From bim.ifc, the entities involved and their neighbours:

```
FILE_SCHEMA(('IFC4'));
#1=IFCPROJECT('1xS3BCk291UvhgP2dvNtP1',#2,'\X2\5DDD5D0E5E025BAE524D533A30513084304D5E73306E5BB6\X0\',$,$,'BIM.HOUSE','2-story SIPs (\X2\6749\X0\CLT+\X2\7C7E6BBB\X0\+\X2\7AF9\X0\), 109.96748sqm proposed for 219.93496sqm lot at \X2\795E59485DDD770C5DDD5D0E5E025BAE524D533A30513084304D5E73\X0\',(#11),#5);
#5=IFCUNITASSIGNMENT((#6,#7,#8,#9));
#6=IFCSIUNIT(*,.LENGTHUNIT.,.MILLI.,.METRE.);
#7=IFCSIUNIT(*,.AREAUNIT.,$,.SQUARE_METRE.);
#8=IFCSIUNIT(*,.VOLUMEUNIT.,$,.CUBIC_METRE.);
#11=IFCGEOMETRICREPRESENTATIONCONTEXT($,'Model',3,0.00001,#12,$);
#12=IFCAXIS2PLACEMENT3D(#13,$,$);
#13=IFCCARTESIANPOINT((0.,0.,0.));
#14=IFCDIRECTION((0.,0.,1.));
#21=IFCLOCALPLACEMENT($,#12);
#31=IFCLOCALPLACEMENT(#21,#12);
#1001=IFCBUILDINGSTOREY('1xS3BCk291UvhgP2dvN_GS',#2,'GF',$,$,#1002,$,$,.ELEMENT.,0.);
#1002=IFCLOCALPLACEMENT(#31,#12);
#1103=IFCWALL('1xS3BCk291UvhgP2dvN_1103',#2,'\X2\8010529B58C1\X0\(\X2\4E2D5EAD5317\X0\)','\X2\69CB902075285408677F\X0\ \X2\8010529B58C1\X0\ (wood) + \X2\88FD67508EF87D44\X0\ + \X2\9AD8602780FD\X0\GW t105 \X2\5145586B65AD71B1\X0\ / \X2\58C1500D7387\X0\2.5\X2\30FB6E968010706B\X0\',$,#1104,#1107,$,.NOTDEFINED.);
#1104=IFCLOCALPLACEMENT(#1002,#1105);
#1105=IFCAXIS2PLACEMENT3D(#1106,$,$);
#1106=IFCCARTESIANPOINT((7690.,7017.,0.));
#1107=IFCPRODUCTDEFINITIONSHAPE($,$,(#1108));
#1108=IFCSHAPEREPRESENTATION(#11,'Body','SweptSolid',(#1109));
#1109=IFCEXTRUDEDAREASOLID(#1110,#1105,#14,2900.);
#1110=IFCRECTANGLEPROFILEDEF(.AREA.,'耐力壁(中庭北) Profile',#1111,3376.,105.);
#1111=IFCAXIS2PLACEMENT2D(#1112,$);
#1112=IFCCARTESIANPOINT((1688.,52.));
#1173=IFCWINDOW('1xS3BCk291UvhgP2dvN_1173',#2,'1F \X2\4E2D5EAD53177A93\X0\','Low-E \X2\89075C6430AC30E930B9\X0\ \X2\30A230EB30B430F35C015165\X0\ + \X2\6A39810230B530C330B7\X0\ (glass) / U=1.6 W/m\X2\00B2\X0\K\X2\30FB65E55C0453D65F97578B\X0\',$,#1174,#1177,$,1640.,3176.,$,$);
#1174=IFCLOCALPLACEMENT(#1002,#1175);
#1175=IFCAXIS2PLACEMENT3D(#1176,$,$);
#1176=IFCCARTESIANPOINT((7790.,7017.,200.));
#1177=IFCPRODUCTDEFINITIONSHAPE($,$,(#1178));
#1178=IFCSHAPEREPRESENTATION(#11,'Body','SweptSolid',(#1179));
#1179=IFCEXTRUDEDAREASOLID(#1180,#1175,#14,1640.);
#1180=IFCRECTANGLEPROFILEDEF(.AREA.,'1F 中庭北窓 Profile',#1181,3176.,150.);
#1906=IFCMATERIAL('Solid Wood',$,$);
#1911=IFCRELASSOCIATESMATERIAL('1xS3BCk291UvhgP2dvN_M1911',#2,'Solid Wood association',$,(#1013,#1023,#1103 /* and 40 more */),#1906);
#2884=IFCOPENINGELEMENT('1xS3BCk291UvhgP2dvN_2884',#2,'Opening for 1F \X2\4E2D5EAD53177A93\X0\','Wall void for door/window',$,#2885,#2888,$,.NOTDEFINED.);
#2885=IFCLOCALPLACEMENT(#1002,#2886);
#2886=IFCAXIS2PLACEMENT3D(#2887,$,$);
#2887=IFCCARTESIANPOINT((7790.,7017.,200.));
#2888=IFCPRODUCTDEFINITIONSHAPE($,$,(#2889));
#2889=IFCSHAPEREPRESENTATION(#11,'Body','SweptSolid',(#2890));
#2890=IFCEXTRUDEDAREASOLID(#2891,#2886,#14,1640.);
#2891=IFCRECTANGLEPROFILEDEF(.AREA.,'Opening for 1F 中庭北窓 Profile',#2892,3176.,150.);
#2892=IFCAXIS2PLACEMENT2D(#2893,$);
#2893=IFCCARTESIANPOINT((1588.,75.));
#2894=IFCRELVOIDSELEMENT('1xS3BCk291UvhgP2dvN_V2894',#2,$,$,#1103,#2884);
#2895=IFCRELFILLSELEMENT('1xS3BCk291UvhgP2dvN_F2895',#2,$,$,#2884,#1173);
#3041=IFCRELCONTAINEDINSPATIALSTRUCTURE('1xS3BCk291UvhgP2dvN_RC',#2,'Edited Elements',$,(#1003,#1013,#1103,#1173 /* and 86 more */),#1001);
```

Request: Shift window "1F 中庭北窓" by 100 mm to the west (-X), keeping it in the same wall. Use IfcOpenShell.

```python
import ifcopenshell
import ifcopenshell.api.geometry
import ifcopenshell.util.placement
import ifcopenshell.util.unit

model = ifcopenshell.open("bim.ifc")
unit_scale = ifcopenshell.util.unit.calculate_unit_scale(model)

window = model.by_guid("1xS3BCk291UvhgP2dvN_1173")
opening = window.FillsVoids[0].RelatingOpeningElement
wall = opening.VoidsElements[0].RelatingBuildingElement

wall_matrix = ifcopenshell.util.placement.get_local_placement(wall.ObjectPlacement)
shift = wall_matrix[:3, 0] * -0.1 / unit_scale
before = ifcopenshell.util.placement.get_local_placement(window.ObjectPlacement)[:3, 3].copy()

# The window is not placed relative to its opening, so move both.
for product in (opening, window):
    matrix = ifcopenshell.util.placement.get_local_placement(product.ObjectPlacement)
    matrix[:3, 3] += shift
    ifcopenshell.api.geometry.edit_object_placement(model, product=product, matrix=matrix, is_si=False)

after = ifcopenshell.util.placement.get_local_placement(window.ObjectPlacement)[:3, 3]
print("window moved by", (after - before).round(3) + 0.0)

model.write("bim_v2.ifc")
```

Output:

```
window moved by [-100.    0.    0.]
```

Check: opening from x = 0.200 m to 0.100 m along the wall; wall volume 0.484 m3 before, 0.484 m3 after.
